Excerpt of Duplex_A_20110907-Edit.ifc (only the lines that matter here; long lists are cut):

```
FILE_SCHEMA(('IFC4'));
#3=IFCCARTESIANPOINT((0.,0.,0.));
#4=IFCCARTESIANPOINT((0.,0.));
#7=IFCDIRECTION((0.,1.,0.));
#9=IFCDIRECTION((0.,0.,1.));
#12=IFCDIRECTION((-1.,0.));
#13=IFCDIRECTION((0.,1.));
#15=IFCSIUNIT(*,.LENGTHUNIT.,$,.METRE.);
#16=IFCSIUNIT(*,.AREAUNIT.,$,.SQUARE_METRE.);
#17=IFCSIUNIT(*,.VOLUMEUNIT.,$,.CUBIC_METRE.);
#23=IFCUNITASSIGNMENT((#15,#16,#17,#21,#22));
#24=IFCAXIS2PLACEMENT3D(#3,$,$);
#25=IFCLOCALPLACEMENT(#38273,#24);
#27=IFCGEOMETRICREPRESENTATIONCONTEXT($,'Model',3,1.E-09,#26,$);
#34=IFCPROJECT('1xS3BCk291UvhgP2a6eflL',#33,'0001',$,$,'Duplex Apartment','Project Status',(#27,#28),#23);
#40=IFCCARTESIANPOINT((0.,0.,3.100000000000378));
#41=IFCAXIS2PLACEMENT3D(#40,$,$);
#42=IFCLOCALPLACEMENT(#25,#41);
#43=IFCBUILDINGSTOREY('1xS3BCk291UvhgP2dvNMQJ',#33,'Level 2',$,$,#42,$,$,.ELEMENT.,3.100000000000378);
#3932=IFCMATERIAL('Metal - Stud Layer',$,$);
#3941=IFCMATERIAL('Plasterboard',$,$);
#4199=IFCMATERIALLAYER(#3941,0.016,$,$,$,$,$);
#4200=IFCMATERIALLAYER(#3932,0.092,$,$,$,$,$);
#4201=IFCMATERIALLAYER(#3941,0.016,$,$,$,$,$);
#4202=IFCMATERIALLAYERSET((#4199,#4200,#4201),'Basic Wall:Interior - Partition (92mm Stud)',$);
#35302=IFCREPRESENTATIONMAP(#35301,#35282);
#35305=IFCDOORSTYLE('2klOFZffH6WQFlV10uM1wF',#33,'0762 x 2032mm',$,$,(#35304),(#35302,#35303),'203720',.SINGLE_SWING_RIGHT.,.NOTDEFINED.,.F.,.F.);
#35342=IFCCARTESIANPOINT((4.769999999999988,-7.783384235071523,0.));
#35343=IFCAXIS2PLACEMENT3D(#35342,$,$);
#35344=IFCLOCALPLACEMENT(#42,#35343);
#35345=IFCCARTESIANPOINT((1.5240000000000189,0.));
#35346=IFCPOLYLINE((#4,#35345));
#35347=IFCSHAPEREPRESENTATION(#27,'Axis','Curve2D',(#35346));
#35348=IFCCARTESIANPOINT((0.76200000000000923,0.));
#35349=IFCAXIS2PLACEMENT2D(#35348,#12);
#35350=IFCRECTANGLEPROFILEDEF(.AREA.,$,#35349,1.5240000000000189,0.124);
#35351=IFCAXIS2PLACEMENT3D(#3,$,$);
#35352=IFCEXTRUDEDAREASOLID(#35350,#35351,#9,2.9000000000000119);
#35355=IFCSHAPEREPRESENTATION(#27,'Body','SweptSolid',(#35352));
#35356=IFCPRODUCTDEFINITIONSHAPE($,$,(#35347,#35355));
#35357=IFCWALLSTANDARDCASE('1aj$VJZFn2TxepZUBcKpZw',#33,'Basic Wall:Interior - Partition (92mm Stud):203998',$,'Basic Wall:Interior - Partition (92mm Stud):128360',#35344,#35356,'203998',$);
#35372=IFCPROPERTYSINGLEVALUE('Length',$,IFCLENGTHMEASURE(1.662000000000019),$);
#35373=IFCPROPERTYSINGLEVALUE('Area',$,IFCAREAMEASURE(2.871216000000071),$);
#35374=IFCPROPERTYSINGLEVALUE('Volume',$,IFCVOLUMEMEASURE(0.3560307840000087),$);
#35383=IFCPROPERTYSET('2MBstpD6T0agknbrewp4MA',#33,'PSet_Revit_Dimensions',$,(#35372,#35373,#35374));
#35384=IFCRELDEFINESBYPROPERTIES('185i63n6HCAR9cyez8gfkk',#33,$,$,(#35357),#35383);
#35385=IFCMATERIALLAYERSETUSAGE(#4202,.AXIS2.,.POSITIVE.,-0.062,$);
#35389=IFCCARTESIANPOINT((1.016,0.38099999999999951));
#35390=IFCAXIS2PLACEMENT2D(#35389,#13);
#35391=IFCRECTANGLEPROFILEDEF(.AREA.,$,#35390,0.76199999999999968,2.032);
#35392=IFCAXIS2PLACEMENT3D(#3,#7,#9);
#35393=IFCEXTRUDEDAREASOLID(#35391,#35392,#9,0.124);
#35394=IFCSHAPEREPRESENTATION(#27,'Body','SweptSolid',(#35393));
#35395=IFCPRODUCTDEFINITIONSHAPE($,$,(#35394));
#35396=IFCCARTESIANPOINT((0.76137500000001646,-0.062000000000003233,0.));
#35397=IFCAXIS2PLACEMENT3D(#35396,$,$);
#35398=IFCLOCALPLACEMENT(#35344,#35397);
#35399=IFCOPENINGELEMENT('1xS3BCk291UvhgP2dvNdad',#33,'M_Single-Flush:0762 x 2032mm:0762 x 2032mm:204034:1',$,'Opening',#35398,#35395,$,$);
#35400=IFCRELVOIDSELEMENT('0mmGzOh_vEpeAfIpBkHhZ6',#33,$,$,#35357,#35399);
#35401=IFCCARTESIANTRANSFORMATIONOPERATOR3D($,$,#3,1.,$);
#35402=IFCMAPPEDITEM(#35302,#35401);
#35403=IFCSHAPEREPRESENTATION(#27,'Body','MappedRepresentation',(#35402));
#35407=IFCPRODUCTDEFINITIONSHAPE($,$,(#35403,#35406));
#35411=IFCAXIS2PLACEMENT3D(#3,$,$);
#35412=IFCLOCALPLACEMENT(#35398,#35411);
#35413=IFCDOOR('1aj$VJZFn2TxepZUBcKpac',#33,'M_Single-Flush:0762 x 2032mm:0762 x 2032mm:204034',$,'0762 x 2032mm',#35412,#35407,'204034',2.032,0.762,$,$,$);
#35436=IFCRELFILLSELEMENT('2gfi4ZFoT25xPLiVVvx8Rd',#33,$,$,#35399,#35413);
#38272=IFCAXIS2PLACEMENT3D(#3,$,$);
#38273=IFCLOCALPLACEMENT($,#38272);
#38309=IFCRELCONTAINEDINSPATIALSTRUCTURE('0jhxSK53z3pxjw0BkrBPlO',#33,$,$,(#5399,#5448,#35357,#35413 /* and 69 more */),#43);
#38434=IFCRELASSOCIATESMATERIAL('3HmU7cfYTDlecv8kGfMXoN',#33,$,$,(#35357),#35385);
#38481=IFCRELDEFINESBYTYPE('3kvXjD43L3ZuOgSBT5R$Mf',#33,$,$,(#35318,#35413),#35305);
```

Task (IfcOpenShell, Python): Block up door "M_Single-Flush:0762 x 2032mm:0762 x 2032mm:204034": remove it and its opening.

```python
import ifcopenshell
import ifcopenshell.api.feature
import ifcopenshell.api.pset
import ifcopenshell.api.root
import ifcopenshell.geom
import ifcopenshell.util.element
import ifcopenshell.util.shape
import ifcopenshell.util.unit

model = ifcopenshell.open("Duplex_A_20110907-Edit.ifc")
area_scale = ifcopenshell.util.unit.calculate_unit_scale(model, "AREAUNIT")
volume_scale = ifcopenshell.util.unit.calculate_unit_scale(model, "VOLUMEUNIT")
settings = ifcopenshell.geom.settings()


def volume(element):
    """Net volume in cubic metres, openings subtracted."""
    shape = ifcopenshell.geom.create_shape(settings, element)
    return ifcopenshell.util.shape.get_volume(shape.geometry)


door = model.by_id(35413)
opening = door.FillsVoids[0].RelatingOpeningElement
wall = opening.VoidsElements[0].RelatingBuildingElement
before = volume(wall)

ifcopenshell.api.root.remove_product(model, product=door)
ifcopenshell.api.feature.remove_feature(model, feature=opening)

after = volume(wall)
thickness = 0.124  # wall thickness in metres

# Update the wall's stored quantities.
pset = model.by_id(ifcopenshell.util.element.get_pset(wall, "PSet_Revit_Dimensions", should_inherit=False)["id"])
ifcopenshell.api.pset.edit_pset(model, pset=pset, properties={
    "Area": model.create_entity("IfcAreaMeasure", after / thickness / area_scale),
    "Volume": model.create_entity("IfcVolumeMeasure", after / volume_scale),
})

print(f"wall volume {before:.3f} -> {after:.3f} m3")

model.write("Duplex_A_20110907-Edit_updated.ifc")
```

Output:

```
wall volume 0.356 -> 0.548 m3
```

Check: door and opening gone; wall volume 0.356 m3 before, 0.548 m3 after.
